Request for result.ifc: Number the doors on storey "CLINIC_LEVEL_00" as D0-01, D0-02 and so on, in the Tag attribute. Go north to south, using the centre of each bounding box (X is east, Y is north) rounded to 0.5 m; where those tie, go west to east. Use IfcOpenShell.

First a look at what the model holds.

```python
import ifcopenshell
import ifcopenshell.util.element
import ifcopenshell.util.placement

model = ifcopenshell.open("result.ifc")
print(model.schema)
storey = next(s for s in model.by_type("IfcBuildingStorey") if s.Name == "CLINIC_LEVEL_00")
doors = [e for e in ifcopenshell.util.element.get_decomposition(storey) if e.is_a("IfcDoor")]
for e in sorted(doors, key=lambda e: e.id()):
    origin = ifcopenshell.util.placement.get_local_placement(e.ObjectPlacement)[:3, 3]
    print(e.id(), e.Tag, e.Name, origin.round(2) + 0.0, sep=" | ")
```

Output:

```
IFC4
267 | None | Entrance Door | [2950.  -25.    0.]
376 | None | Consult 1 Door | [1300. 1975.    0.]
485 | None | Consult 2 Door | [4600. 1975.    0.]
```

```python
import ifcopenshell
import ifcopenshell.geom
import ifcopenshell.util.element
import ifcopenshell.util.shape

model = ifcopenshell.open("result.ifc")
settings = ifcopenshell.geom.settings()
settings.set("use-world-coords", True)


def centre(element):
    shape = ifcopenshell.geom.create_shape(settings, element)
    return ifcopenshell.util.shape.get_bbox_centroid(shape.geometry)


storey = next(s for s in model.by_type("IfcBuildingStorey") if s.Name == "CLINIC_LEVEL_00")
doors = [e for e in ifcopenshell.util.element.get_decomposition(storey) if e.is_a("IfcDoor")]

# Insertion points can sit at a corner or the storey origin, so sort by the geometry (in metres).
centres = {e: centre(e) for e in doors}
doors.sort(key=lambda e: (-round(centres[e][1] / 0.5), centres[e][0]))

for i, e in enumerate(doors, start=1):
    number = f"D0-{i:02d}"
    e.Tag = number
    print(e.id(), number)

model.write("result-out.ifc")
```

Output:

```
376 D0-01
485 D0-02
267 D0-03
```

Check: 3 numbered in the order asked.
